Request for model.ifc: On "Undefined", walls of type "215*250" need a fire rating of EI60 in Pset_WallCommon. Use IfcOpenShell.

First a look at what the model holds.

```python
import ifcopenshell
import ifcopenshell.util.element

model = ifcopenshell.open("model.ifc")
print(model.schema)
storey = next(s for s in model.by_type("IfcBuildingStorey") if s.Name == "Undefined")
walls = [e for e in ifcopenshell.util.element.get_decomposition(storey) if e.is_a("IfcWall")]
seen = {}
for e in walls:
    element_type = ifcopenshell.util.element.get_type(e)
    key = (element_type.Name if element_type != e and element_type else None, ifcopenshell.util.element.get_pset(e, "Pset_WallCommon", "FireRating"))
    seen[key] = seen.get(key, 0) + 1
for (name, value), count in sorted(seen.items(), key=str):
    print(count, "x", name, "|", value)
```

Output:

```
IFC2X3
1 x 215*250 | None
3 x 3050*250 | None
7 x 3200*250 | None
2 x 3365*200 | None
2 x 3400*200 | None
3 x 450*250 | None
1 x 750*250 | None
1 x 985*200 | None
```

```python
import ifcopenshell
import ifcopenshell.api.pset
import ifcopenshell.util.element

model = ifcopenshell.open("model.ifc")

storey = next(s for s in model.by_type("IfcBuildingStorey") if s.Name == "Undefined")
walls = [e for e in ifcopenshell.util.element.get_decomposition(storey) if e.is_a("IfcWall")]

count = 0
for e in walls:
    element_type = ifcopenshell.util.element.get_type(e)
    if element_type in (None, e) or element_type.Name != "215*250":
        continue
    # add_pset returns the element's existing set when there is one.
    pset = ifcopenshell.api.pset.add_pset(model, product=e, name="Pset_WallCommon")
    ifcopenshell.api.pset.edit_pset(model, pset=pset, properties={"FireRating": "EI60"})
    count += 1

print(count, "walls updated")

model.write("model_edited.ifc")
```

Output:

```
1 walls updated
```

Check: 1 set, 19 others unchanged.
